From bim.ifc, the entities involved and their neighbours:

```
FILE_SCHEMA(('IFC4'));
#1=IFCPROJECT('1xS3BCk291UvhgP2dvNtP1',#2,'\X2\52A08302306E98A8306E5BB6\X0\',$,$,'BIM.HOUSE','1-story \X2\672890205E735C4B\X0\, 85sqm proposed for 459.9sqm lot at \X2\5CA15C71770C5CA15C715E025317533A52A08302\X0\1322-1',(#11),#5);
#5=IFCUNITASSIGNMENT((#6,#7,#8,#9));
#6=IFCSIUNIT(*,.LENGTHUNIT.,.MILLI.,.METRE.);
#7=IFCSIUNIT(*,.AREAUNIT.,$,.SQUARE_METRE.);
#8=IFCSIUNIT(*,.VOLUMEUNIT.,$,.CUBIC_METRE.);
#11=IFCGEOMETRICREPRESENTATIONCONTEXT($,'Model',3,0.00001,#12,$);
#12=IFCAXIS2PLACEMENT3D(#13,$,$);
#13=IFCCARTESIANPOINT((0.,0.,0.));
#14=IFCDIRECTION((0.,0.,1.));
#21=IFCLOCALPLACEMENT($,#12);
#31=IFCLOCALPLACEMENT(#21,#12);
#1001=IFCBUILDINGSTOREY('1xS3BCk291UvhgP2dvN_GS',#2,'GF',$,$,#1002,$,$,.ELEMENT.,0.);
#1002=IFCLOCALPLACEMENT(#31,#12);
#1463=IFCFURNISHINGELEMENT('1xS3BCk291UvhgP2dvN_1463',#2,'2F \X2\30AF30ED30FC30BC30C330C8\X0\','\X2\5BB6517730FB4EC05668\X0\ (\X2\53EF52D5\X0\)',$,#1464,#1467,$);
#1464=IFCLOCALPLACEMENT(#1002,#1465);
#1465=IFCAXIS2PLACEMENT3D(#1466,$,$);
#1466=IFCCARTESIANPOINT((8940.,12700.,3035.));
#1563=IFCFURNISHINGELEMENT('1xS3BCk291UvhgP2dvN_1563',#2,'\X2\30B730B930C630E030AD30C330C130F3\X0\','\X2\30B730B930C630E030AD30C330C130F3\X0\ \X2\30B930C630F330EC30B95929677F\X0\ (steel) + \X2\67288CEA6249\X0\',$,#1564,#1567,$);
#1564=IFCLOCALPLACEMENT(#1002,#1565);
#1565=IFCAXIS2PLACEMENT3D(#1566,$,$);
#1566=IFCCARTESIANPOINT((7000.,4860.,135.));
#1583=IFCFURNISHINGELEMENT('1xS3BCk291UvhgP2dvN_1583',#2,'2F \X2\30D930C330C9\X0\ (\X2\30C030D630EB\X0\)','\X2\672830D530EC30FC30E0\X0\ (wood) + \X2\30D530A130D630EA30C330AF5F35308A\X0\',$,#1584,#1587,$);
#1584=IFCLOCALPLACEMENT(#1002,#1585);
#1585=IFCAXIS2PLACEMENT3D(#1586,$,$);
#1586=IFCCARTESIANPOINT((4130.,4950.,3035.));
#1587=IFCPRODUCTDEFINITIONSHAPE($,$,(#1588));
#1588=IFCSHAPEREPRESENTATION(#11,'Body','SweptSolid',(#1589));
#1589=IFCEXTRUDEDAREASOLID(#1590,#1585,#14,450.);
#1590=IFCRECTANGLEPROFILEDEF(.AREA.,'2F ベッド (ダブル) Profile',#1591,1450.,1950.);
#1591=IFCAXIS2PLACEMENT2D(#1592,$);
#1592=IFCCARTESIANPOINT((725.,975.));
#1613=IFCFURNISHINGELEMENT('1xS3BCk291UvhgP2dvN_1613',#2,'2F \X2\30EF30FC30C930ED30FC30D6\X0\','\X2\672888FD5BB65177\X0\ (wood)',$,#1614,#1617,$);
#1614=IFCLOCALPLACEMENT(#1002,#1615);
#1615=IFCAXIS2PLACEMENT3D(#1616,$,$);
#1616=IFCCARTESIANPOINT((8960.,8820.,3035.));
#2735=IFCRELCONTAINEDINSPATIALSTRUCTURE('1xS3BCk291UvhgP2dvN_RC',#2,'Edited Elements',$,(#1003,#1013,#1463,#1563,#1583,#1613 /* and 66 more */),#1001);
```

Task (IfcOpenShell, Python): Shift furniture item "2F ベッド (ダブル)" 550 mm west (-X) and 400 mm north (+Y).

```python
import ifcopenshell
import ifcopenshell.api.geometry
import ifcopenshell.util.placement

model = ifcopenshell.open("bim.ifc")

item = model.by_guid("1xS3BCk291UvhgP2dvN_1583")
matrix = ifcopenshell.util.placement.get_local_placement(item.ObjectPlacement)
matrix[0, 3] -= 550.0
matrix[1, 3] += 400.0
ifcopenshell.api.geometry.edit_object_placement(model, product=item, matrix=matrix, is_si=False)

print(ifcopenshell.util.placement.get_local_placement(item.ObjectPlacement).round(3) + 0.0)

model.write("bim_rev.ifc")
```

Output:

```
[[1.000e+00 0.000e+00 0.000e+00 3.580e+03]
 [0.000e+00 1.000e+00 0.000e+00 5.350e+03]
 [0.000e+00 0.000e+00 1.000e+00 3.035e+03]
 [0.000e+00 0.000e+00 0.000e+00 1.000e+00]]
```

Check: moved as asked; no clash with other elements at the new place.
